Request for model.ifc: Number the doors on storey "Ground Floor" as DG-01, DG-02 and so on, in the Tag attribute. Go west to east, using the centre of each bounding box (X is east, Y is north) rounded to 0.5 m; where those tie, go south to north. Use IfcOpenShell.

First a look at what the model holds.

```python
import ifcopenshell
import ifcopenshell.util.element
import ifcopenshell.util.placement

model = ifcopenshell.open("model.ifc")
print(model.schema)
storey = next(s for s in model.by_type("IfcBuildingStorey") if s.Name == "Ground Floor")
doors = [e for e in ifcopenshell.util.element.get_decomposition(storey) if e.is_a("IfcDoor")]
for e in sorted(doors, key=lambda e: e.id()):
    origin = ifcopenshell.util.placement.get_local_placement(e.ObjectPlacement)[:3, 3]
    print(e.id(), e.Tag, e.Name, origin.round(2) + 0.0, sep=" | ")
```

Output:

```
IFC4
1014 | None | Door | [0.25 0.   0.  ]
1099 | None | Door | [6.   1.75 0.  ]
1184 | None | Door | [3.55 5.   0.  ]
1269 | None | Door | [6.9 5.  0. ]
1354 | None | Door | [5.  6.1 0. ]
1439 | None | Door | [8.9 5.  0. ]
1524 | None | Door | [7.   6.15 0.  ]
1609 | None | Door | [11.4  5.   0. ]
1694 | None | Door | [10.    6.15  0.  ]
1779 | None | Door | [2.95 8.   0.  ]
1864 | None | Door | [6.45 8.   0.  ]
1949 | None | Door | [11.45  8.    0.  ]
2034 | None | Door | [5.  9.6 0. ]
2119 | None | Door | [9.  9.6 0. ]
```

```python
import ifcopenshell
import ifcopenshell.geom
import ifcopenshell.util.element
import ifcopenshell.util.shape

model = ifcopenshell.open("model.ifc")
settings = ifcopenshell.geom.settings()
settings.set("use-world-coords", True)


def centre(element):
    shape = ifcopenshell.geom.create_shape(settings, element)
    return ifcopenshell.util.shape.get_bbox_centroid(shape.geometry)


storey = next(s for s in model.by_type("IfcBuildingStorey") if s.Name == "Ground Floor")
doors = [e for e in ifcopenshell.util.element.get_decomposition(storey) if e.is_a("IfcDoor")]

# Insertion points can sit at a corner or the storey origin, so sort by the geometry (in metres).
centres = {e: centre(e) for e in doors}
doors.sort(key=lambda e: (round(centres[e][0] / 0.5), centres[e][1]))

for i, e in enumerate(doors, start=1):
    number = f"DG-{i:02d}"
    e.Tag = number
    print(e.id(), number)

model.write("model_updated.ifc")
```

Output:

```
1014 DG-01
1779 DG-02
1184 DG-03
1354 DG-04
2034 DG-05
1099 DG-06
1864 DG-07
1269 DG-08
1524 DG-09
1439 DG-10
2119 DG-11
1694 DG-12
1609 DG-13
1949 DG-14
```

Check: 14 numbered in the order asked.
